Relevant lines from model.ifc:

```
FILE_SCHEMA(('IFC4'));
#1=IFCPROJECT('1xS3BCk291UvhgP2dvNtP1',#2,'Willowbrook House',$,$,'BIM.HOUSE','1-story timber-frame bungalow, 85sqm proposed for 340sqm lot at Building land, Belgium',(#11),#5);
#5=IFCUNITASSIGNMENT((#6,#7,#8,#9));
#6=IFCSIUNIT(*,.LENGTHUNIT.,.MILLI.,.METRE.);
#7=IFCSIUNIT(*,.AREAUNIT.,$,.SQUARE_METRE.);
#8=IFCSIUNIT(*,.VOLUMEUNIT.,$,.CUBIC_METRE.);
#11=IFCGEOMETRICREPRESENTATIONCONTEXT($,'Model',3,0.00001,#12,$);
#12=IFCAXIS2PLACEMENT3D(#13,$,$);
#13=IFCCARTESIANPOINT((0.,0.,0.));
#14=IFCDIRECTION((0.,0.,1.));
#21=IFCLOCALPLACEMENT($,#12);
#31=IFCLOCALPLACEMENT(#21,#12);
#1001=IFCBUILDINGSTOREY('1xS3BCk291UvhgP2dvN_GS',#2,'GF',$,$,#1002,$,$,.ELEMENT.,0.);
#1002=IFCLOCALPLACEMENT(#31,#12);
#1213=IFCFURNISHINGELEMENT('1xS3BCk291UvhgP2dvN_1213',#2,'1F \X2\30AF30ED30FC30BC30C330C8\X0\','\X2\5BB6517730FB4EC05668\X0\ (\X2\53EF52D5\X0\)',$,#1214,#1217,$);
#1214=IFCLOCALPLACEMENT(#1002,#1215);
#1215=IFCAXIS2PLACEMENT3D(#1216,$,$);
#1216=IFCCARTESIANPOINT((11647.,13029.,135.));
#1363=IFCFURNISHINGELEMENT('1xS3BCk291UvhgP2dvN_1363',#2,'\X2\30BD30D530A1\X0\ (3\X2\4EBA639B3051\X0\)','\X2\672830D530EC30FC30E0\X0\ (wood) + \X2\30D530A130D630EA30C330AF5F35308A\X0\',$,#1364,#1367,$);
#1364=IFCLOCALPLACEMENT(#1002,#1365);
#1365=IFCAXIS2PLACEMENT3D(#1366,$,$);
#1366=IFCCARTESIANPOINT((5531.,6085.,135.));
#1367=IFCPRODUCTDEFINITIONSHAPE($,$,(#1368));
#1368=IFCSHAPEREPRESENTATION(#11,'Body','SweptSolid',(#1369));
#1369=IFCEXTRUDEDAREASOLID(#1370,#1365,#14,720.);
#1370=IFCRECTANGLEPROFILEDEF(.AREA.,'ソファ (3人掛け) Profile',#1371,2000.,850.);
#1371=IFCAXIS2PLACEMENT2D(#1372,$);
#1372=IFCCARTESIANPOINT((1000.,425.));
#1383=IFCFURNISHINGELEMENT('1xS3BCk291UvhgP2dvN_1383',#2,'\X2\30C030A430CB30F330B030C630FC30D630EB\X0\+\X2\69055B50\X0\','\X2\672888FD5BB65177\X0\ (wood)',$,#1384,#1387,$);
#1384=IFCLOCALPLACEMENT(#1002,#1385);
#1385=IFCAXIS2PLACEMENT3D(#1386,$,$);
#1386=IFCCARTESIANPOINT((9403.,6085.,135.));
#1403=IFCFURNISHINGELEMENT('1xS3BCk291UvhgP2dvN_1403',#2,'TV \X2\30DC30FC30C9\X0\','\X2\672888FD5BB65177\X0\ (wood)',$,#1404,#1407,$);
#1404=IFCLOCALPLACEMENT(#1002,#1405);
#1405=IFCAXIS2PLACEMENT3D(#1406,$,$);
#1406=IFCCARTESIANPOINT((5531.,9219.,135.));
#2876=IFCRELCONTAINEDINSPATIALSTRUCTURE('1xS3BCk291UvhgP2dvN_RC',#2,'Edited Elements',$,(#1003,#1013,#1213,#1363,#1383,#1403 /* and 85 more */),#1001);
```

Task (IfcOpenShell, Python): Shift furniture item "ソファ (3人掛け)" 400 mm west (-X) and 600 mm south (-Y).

```python
import ifcopenshell
import ifcopenshell.api.geometry
import ifcopenshell.util.placement

model = ifcopenshell.open("model.ifc")

item = model.by_id(1363)
matrix = ifcopenshell.util.placement.get_local_placement(item.ObjectPlacement)
matrix[0, 3] -= 400.0
matrix[1, 3] -= 600.0
ifcopenshell.api.geometry.edit_object_placement(model, product=item, matrix=matrix, is_si=False)

print(ifcopenshell.util.placement.get_local_placement(item.ObjectPlacement).round(3) + 0.0)

model.write("model_updated.ifc")
```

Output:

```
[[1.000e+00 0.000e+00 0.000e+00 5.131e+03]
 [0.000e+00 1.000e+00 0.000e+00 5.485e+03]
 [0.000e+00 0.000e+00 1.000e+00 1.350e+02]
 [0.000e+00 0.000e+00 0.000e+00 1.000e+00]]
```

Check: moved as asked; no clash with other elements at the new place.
